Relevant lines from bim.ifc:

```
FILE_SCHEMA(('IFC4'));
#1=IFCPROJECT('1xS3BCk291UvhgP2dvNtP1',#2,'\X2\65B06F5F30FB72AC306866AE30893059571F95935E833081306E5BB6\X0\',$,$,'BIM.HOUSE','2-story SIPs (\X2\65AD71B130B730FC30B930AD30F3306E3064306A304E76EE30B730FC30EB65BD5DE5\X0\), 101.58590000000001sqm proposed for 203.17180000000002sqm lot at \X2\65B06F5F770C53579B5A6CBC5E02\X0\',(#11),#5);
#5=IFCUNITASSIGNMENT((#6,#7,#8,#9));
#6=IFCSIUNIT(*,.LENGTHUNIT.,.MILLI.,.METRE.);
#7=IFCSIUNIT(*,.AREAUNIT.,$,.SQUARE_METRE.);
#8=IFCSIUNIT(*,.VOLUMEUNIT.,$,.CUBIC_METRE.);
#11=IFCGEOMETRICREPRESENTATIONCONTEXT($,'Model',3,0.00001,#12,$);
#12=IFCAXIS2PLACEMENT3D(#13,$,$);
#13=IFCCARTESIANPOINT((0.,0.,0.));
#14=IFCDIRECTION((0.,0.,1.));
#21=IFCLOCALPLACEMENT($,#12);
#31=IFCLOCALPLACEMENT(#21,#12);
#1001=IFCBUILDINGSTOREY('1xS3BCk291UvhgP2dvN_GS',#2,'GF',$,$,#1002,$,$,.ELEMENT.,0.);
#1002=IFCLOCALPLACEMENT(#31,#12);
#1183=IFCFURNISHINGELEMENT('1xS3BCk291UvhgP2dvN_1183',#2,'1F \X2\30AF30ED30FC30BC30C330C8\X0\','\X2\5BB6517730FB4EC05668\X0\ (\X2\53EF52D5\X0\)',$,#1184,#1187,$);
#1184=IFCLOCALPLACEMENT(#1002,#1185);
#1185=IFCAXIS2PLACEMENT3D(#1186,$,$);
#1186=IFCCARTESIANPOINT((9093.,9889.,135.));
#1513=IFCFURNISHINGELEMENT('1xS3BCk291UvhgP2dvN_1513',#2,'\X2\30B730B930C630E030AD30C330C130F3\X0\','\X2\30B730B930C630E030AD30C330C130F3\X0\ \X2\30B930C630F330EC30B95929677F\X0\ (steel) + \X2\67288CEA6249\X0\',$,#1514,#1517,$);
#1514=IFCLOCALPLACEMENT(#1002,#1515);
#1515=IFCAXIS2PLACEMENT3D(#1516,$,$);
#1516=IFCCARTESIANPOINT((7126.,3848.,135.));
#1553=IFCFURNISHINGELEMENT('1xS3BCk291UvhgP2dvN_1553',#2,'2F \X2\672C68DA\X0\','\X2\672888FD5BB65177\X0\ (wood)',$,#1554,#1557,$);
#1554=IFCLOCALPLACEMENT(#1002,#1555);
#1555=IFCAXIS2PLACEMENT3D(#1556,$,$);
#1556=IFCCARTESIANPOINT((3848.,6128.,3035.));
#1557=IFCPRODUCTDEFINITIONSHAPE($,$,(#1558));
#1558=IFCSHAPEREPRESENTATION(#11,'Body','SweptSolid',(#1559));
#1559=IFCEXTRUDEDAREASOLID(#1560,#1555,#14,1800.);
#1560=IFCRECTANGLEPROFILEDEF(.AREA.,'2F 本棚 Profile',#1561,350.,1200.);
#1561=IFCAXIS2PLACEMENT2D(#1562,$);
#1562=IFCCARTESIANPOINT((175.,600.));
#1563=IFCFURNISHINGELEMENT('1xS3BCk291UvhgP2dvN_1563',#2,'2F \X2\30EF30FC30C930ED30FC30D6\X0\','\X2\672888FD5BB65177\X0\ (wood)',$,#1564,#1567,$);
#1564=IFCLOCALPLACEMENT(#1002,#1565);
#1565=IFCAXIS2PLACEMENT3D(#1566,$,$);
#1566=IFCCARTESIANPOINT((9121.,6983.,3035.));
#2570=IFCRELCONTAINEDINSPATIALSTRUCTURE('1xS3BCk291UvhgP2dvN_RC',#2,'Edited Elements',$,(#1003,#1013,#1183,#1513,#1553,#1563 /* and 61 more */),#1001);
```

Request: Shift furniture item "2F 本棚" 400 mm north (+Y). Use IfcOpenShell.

```python
import ifcopenshell
import ifcopenshell.api.geometry
import ifcopenshell.util.placement
import ifcopenshell.util.unit

model = ifcopenshell.open("bim.ifc")
unit_scale = ifcopenshell.util.unit.calculate_unit_scale(model)

item = model.by_guid("1xS3BCk291UvhgP2dvN_1553")
matrix = ifcopenshell.util.placement.get_local_placement(item.ObjectPlacement)
matrix[1, 3] += 0.4 / unit_scale
ifcopenshell.api.geometry.edit_object_placement(model, product=item, matrix=matrix, is_si=False)

print(ifcopenshell.util.placement.get_local_placement(item.ObjectPlacement).round(3) + 0.0)

model.write("bim_edited.ifc")
```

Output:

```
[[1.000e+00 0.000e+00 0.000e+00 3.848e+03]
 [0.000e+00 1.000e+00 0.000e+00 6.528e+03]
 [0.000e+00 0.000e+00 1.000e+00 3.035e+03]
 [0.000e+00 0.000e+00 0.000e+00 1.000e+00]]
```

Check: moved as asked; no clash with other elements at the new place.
